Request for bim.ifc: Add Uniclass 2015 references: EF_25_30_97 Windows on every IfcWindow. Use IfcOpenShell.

First a look at what the model holds.

```python
import ifcopenshell

model = ifcopenshell.open("bim.ifc")
print(model.schema)
print("classifications:", [c.Name for c in model.by_type("IfcClassification")])
for ifc_class in ("IfcDoor", "IfcRoof", "IfcStair", "IfcWall", "IfcWindow"):
    print(ifc_class, len(model.by_type(ifc_class)))
```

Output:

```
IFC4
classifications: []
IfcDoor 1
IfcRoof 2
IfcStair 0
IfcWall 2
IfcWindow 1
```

```python
import ifcopenshell
import ifcopenshell.api.classification

model = ifcopenshell.open("bim.ifc")

system = ifcopenshell.api.classification.add_classification(model, classification="Uniclass 2015")

codes = {
    "IfcWindow": ("EF_25_30_97", "Windows"),
}
for ifc_class, (code, name) in codes.items():
    products = model.by_type(ifc_class)
    ifcopenshell.api.classification.add_reference(
        model, products=products, classification=system, identification=code, name=name
    )
    print(code, len(products))

model.write("bim-out.ifc")
```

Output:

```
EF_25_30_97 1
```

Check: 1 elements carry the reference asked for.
